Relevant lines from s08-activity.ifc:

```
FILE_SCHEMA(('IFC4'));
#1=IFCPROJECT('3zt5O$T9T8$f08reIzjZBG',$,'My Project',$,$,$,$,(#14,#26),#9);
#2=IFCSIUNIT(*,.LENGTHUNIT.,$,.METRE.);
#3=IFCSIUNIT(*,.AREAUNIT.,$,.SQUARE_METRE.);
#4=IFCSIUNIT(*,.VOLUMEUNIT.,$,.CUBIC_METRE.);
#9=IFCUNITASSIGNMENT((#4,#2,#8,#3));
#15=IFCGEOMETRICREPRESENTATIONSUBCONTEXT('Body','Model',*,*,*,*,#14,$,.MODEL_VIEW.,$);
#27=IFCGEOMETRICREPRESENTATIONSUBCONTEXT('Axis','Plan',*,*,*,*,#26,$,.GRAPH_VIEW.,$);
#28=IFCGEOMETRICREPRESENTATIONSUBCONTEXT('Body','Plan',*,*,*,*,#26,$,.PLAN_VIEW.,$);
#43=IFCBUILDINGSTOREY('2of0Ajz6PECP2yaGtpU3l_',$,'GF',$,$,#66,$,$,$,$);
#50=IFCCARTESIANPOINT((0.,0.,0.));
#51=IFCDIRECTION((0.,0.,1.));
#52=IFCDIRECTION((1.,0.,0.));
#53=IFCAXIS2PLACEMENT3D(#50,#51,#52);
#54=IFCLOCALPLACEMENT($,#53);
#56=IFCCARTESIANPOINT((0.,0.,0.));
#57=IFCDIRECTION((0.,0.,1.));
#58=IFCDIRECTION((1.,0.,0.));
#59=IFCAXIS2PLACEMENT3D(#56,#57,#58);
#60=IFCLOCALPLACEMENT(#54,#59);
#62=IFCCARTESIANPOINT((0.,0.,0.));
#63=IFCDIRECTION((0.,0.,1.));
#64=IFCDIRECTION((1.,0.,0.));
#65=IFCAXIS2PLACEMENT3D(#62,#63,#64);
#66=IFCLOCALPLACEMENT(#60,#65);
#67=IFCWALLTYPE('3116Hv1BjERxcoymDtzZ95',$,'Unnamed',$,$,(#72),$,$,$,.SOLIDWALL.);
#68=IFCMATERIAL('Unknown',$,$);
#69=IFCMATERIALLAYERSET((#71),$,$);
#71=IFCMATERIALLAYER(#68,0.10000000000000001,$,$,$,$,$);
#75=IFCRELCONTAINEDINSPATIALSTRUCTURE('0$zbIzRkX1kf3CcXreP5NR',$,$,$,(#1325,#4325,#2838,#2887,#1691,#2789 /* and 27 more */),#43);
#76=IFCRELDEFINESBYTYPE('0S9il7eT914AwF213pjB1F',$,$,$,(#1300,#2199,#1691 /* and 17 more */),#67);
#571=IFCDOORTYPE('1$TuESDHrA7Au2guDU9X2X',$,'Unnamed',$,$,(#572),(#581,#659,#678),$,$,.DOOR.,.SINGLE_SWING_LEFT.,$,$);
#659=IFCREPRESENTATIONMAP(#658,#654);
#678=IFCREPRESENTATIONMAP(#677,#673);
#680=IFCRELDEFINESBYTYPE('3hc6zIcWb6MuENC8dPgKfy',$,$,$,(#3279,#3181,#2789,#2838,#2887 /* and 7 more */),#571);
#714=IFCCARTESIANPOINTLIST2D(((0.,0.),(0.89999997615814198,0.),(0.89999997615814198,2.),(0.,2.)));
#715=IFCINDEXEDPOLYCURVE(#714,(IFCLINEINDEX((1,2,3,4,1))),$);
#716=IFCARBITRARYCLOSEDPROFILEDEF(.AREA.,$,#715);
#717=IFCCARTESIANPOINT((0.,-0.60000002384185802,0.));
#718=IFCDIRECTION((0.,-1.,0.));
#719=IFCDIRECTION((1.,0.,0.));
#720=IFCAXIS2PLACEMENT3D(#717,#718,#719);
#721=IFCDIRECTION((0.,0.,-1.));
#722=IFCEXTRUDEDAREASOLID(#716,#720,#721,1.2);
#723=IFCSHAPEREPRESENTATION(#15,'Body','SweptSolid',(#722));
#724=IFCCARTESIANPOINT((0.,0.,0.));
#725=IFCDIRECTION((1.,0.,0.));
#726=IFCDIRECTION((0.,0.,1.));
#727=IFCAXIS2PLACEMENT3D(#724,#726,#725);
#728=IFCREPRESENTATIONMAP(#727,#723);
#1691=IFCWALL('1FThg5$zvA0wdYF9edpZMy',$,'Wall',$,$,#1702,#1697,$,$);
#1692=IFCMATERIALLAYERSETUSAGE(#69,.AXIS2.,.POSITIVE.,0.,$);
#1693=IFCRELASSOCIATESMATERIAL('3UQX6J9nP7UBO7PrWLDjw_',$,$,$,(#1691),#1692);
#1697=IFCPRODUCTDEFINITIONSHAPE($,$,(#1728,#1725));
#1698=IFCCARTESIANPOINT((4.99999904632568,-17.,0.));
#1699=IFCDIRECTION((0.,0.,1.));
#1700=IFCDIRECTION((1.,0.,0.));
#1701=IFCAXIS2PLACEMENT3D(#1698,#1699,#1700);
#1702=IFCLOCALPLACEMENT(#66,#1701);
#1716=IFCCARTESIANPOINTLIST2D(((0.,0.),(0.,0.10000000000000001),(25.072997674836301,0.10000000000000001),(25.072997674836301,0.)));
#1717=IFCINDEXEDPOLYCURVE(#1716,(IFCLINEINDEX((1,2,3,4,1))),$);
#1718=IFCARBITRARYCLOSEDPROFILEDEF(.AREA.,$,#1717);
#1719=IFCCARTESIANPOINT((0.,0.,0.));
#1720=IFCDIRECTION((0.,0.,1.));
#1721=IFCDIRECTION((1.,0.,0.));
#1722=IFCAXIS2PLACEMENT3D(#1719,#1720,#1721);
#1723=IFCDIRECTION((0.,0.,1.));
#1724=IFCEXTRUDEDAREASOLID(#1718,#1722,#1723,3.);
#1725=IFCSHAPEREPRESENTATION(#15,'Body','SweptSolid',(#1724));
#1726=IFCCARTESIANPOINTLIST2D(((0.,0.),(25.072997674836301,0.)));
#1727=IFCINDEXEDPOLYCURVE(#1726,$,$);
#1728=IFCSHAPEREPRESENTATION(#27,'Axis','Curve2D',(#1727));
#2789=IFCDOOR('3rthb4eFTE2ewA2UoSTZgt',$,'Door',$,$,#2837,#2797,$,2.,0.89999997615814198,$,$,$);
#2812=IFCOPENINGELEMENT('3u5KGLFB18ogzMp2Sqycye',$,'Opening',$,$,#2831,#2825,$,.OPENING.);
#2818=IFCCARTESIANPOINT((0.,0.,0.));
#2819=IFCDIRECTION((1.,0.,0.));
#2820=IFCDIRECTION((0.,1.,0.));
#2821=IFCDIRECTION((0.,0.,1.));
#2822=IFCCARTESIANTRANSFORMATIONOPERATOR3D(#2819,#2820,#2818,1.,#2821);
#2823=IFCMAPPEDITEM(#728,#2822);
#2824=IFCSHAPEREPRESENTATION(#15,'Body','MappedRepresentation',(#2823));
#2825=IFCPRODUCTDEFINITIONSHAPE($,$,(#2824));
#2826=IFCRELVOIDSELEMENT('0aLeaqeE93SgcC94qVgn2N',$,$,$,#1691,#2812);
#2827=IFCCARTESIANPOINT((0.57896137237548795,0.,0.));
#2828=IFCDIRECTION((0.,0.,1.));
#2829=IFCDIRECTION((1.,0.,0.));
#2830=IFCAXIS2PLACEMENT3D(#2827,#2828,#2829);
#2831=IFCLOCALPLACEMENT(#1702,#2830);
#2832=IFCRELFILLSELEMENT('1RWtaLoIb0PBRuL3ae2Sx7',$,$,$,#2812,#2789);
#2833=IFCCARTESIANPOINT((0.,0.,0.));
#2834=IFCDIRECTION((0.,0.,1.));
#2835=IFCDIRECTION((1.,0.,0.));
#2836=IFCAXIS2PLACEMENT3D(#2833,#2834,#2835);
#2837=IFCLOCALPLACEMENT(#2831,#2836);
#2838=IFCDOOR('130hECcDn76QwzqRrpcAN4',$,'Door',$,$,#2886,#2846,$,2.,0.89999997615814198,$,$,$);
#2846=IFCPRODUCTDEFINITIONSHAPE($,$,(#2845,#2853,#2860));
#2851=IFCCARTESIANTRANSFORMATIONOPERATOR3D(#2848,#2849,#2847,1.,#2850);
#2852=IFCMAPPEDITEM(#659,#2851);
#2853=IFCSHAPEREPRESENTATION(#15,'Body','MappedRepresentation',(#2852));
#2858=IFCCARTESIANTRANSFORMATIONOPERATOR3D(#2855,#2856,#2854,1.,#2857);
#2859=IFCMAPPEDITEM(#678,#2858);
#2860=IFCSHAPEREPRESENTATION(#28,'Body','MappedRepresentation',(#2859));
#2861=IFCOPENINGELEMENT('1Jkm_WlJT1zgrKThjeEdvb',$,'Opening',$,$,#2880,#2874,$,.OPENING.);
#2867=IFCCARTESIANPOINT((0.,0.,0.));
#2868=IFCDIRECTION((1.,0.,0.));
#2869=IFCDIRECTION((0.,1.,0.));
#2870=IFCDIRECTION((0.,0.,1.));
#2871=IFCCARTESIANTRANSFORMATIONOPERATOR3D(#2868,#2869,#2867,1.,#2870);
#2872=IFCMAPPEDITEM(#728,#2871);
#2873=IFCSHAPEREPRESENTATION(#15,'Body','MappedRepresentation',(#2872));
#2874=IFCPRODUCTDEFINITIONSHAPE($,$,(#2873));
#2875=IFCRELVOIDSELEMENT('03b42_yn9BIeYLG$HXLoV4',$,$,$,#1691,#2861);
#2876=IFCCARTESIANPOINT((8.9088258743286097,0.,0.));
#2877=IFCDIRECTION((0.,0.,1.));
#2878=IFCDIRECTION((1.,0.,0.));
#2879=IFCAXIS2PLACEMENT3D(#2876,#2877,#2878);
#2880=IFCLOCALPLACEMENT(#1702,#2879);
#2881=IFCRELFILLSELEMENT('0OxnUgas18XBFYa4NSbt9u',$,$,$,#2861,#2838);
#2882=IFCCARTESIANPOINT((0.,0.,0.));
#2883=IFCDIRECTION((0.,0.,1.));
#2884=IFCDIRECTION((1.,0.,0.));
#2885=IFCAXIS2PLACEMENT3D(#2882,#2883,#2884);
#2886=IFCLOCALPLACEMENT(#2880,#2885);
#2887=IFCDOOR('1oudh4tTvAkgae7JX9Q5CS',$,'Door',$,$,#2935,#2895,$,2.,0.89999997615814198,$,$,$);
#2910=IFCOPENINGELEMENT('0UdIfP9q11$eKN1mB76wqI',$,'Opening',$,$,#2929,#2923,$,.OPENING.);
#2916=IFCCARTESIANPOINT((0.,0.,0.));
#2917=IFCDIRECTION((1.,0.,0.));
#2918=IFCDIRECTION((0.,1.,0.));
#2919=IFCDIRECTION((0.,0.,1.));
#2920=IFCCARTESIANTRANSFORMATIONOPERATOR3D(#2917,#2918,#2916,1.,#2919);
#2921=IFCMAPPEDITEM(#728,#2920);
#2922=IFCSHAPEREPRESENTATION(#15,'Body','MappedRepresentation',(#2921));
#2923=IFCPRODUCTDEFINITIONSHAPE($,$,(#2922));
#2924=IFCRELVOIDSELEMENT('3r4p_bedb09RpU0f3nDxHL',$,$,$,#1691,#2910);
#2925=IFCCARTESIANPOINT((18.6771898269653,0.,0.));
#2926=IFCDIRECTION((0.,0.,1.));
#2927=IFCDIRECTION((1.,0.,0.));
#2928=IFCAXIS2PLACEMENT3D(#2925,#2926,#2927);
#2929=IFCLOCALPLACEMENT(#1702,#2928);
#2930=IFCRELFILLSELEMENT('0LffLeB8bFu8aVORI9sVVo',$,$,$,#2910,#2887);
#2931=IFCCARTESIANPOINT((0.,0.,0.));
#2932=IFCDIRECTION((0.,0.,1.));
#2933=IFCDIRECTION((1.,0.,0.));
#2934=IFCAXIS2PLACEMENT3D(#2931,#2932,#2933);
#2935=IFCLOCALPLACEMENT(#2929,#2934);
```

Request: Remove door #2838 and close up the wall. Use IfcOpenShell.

```python
import ifcopenshell
import ifcopenshell.api.feature
import ifcopenshell.api.root
import ifcopenshell.geom
import ifcopenshell.util.shape

model = ifcopenshell.open("s08-activity.ifc")
settings = ifcopenshell.geom.settings()


def volume(element):
    """Net volume in cubic metres, openings subtracted."""
    shape = ifcopenshell.geom.create_shape(settings, element)
    return ifcopenshell.util.shape.get_volume(shape.geometry)


door = model.by_guid("130hECcDn76QwzqRrpcAN4")
opening = door.FillsVoids[0].RelatingOpeningElement
wall = opening.VoidsElements[0].RelatingBuildingElement
before = volume(wall)

ifcopenshell.api.root.remove_product(model, product=door)
ifcopenshell.api.feature.remove_feature(model, feature=opening)

after = volume(wall)

print(f"wall volume {before:.3f} -> {after:.3f} m3")

model.write("s08-activity-out.ifc")
```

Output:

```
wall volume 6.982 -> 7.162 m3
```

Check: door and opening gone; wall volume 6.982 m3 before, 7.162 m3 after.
